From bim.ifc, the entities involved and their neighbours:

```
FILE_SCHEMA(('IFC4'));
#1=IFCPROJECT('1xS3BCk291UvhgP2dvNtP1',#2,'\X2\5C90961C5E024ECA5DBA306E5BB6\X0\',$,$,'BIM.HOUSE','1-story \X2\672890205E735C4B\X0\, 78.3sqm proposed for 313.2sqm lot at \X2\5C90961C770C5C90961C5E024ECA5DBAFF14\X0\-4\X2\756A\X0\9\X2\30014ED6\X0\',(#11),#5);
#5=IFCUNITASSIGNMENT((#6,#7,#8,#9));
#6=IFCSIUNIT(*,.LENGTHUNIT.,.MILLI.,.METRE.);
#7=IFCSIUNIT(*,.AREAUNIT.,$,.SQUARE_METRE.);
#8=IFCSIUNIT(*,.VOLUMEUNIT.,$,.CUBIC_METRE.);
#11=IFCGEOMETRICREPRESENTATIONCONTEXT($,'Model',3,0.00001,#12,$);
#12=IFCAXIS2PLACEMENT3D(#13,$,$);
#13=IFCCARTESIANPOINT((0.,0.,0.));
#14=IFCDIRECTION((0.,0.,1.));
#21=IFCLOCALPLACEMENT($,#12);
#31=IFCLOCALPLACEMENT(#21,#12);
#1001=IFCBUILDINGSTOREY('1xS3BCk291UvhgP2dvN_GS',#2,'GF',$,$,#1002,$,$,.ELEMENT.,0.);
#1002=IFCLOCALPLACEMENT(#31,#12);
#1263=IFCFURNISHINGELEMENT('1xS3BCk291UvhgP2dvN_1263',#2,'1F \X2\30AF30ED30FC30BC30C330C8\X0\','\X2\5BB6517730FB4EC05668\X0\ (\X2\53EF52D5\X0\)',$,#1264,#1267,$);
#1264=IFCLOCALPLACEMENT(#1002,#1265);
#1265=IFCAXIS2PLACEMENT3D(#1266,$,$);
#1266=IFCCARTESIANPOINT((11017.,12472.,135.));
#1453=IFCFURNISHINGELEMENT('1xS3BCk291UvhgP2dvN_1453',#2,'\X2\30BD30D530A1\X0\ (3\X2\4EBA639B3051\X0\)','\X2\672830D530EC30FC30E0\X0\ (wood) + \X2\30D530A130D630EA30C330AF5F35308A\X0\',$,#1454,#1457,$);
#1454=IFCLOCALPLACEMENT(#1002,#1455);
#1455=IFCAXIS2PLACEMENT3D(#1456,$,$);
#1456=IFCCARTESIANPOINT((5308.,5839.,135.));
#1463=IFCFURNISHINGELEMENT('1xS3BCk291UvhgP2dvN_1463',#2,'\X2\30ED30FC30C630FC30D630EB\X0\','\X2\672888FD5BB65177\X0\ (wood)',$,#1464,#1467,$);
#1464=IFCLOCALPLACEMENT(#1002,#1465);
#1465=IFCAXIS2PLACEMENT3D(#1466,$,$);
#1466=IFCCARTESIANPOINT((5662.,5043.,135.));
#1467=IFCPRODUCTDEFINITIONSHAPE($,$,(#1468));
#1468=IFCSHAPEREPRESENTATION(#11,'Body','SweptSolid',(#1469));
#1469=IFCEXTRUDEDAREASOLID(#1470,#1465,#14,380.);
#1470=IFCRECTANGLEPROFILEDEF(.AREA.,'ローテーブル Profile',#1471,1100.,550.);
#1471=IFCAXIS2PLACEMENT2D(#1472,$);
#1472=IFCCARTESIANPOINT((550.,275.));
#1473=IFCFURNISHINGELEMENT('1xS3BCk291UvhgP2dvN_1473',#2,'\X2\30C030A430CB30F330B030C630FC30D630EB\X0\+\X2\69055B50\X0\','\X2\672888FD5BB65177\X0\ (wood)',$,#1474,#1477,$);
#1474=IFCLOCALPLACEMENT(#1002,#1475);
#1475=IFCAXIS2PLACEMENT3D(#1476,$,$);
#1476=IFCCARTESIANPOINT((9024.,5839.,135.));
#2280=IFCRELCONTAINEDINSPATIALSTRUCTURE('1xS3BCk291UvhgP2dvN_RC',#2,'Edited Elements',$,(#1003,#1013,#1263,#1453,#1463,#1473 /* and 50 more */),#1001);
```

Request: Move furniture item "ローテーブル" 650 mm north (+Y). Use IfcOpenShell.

```python
import ifcopenshell
import ifcopenshell.api.geometry
import ifcopenshell.util.placement

model = ifcopenshell.open("bim.ifc")

item = model.by_guid("1xS3BCk291UvhgP2dvN_1463")
matrix = ifcopenshell.util.placement.get_local_placement(item.ObjectPlacement)
matrix[1, 3] += 650.0
ifcopenshell.api.geometry.edit_object_placement(model, product=item, matrix=matrix, is_si=False)

print(ifcopenshell.util.placement.get_local_placement(item.ObjectPlacement).round(3) + 0.0)

model.write("bim_updated.ifc")
```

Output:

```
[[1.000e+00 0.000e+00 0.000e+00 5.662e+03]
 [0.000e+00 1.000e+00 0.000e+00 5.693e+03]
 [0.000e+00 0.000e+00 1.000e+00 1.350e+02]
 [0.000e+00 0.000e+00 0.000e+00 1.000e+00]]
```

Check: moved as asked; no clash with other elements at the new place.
